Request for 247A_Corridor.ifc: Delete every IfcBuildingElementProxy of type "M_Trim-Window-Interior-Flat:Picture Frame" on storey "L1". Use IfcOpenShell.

First a look at what the model holds.

```python
import ifcopenshell
import ifcopenshell.util.element

model = ifcopenshell.open("247A_Corridor.ifc")
print(model.schema)
storey = next(s for s in model.by_type("IfcBuildingStorey") if s.Name == "L1")
proxies = [e for e in ifcopenshell.util.element.get_decomposition(storey) if e.is_a("IfcBuildingElementProxy")]
seen = {}
for e in proxies:
    element_type = ifcopenshell.util.element.get_type(e)
    name = element_type.Name if element_type not in (None, e) else None
    seen[name] = seen.get(name, 0) + 1
for name, count in sorted(seen.items(), key=str):
    print(count, "x", name)
```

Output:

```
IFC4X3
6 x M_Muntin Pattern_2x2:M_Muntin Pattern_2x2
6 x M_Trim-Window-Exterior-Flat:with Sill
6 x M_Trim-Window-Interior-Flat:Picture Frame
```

```python
import ifcopenshell
import ifcopenshell.api.root
import ifcopenshell.util.element

model = ifcopenshell.open("247A_Corridor.ifc")

storey = next(s for s in model.by_type("IfcBuildingStorey") if s.Name == "L1")
proxies = [e for e in ifcopenshell.util.element.get_decomposition(storey) if e.is_a("IfcBuildingElementProxy")]
targets = [e for e in proxies if (t := ifcopenshell.util.element.get_type(e)) not in (None, e) and t.Name == "M_Trim-Window-Interior-Flat:Picture Frame"]

for e in targets:
    ifcopenshell.api.root.remove_product(model, product=e)
print(len(targets), "removed")

model.write("247A_Corridor_updated.ifc")
```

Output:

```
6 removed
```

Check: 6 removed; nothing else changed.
